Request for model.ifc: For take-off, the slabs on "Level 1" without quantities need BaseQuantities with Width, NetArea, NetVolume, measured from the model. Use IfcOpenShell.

First a look at what the model holds.

```python
import ifcopenshell
import ifcopenshell.util.element
import ifcopenshell.util.unit

model = ifcopenshell.open("model.ifc")
print(model.schema)
for unit_type in ("LENGTHUNIT", "AREAUNIT", "VOLUMEUNIT"):
    print(unit_type, ifcopenshell.util.unit.calculate_unit_scale(model, unit_type))
storey = next(s for s in model.by_type("IfcBuildingStorey") if s.Name == "Level 1")
slabs = [e for e in ifcopenshell.util.element.get_decomposition(storey) if e.is_a("IfcSlab")]
for e in sorted(slabs, key=lambda e: e.id()):
    print(e.id(), e.is_a(), e.Name, list(ifcopenshell.util.element.get_psets(e, qtos_only=True)), sep=" | ")
```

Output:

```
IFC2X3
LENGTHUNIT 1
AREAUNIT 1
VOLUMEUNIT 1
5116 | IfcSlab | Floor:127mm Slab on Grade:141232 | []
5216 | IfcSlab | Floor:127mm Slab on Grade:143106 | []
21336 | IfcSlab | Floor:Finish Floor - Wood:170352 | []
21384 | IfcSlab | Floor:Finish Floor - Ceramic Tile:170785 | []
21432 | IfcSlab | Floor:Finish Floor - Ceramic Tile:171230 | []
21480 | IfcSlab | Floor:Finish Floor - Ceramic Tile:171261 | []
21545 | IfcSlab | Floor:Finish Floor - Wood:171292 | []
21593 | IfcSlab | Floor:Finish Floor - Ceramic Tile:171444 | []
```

```python
import ifcopenshell
import ifcopenshell.api.pset
import ifcopenshell.geom
import ifcopenshell.util.element
import ifcopenshell.util.shape
import ifcopenshell.util.unit

model = ifcopenshell.open("model.ifc")
unit_scale = ifcopenshell.util.unit.calculate_unit_scale(model)
area_scale = ifcopenshell.util.unit.calculate_unit_scale(model, "AREAUNIT")
volume_scale = ifcopenshell.util.unit.calculate_unit_scale(model, "VOLUMEUNIT")
settings = ifcopenshell.geom.settings()

storey = next(s for s in model.by_type("IfcBuildingStorey") if s.Name == "Level 1")
slabs = [e for e in ifcopenshell.util.element.get_decomposition(storey) if e.is_a("IfcSlab")]

for e in sorted(slabs, key=lambda e: e.id()):
    if ifcopenshell.util.element.get_psets(e, qtos_only=True, should_inherit=False):
        continue
    # Geometry comes back in metres, in the element's own axes.
    shape = ifcopenshell.geom.create_shape(settings, e)
    values = {
        "Width": ifcopenshell.util.shape.get_z(shape.geometry) / unit_scale,
        "NetArea": ifcopenshell.util.shape.get_footprint_area(shape.geometry) / area_scale,
        "NetVolume": ifcopenshell.util.shape.get_volume(shape.geometry) / volume_scale,
    }
    qto = ifcopenshell.api.pset.add_qto(model, product=e, name="BaseQuantities")
    ifcopenshell.api.pset.edit_qto(model, qto=qto, properties=values)
    print(e.id(), {k: round(v, 3) for k, v in values.items()})

model.write("model_v2.ifc")
```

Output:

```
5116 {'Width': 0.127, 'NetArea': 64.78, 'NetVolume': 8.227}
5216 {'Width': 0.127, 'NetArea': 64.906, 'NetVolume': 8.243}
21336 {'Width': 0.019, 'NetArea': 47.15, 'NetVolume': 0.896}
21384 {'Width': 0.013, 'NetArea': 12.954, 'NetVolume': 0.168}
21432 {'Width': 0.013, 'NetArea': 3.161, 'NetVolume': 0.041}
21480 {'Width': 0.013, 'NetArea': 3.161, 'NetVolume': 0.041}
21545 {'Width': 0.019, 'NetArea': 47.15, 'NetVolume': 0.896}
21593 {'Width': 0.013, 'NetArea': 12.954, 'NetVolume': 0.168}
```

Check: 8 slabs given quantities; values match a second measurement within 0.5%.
